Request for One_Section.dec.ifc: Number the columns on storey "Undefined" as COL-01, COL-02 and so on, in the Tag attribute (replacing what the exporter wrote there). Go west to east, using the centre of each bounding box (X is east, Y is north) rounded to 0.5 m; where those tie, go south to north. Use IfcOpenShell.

First a look at what the model holds.

```python
import ifcopenshell
import ifcopenshell.util.element
import ifcopenshell.util.placement

model = ifcopenshell.open("One_Section.dec.ifc")
print(model.schema)
storey = next(s for s in model.by_type("IfcBuildingStorey") if s.Name == "Undefined")
columns = [e for e in ifcopenshell.util.element.get_decomposition(storey) if e.is_a("IfcColumn")]
for e in sorted(columns, key=lambda e: e.id()):
    origin = ifcopenshell.util.placement.get_local_placement(e.ObjectPlacement)[:3, 3]
    print(e.id(), e.Tag, e.Name, origin.round(2) + 0.0, sep=" | ")
```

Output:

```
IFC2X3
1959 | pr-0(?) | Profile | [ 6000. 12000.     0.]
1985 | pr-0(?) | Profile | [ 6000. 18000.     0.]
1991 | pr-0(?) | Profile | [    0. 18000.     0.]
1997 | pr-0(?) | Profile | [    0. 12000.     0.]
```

```python
import ifcopenshell
import ifcopenshell.geom
import ifcopenshell.util.element
import ifcopenshell.util.shape

model = ifcopenshell.open("One_Section.dec.ifc")
settings = ifcopenshell.geom.settings()
settings.set("use-world-coords", True)


def centre(element):
    shape = ifcopenshell.geom.create_shape(settings, element)
    return ifcopenshell.util.shape.get_bbox_centroid(shape.geometry)


storey = next(s for s in model.by_type("IfcBuildingStorey") if s.Name == "Undefined")
columns = [e for e in ifcopenshell.util.element.get_decomposition(storey) if e.is_a("IfcColumn")]

# Insertion points can sit at a corner or the storey origin, so sort by the geometry (in metres).
centres = {e: centre(e) for e in columns}
columns.sort(key=lambda e: (round(centres[e][0] / 0.5), centres[e][1]))

for i, e in enumerate(columns, start=1):
    number = f"COL-{i:02d}"
    e.Tag = number
    print(e.id(), number)

model.write("One_Section.dec_edited.ifc")
```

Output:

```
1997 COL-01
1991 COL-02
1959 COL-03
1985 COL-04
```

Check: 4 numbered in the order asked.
